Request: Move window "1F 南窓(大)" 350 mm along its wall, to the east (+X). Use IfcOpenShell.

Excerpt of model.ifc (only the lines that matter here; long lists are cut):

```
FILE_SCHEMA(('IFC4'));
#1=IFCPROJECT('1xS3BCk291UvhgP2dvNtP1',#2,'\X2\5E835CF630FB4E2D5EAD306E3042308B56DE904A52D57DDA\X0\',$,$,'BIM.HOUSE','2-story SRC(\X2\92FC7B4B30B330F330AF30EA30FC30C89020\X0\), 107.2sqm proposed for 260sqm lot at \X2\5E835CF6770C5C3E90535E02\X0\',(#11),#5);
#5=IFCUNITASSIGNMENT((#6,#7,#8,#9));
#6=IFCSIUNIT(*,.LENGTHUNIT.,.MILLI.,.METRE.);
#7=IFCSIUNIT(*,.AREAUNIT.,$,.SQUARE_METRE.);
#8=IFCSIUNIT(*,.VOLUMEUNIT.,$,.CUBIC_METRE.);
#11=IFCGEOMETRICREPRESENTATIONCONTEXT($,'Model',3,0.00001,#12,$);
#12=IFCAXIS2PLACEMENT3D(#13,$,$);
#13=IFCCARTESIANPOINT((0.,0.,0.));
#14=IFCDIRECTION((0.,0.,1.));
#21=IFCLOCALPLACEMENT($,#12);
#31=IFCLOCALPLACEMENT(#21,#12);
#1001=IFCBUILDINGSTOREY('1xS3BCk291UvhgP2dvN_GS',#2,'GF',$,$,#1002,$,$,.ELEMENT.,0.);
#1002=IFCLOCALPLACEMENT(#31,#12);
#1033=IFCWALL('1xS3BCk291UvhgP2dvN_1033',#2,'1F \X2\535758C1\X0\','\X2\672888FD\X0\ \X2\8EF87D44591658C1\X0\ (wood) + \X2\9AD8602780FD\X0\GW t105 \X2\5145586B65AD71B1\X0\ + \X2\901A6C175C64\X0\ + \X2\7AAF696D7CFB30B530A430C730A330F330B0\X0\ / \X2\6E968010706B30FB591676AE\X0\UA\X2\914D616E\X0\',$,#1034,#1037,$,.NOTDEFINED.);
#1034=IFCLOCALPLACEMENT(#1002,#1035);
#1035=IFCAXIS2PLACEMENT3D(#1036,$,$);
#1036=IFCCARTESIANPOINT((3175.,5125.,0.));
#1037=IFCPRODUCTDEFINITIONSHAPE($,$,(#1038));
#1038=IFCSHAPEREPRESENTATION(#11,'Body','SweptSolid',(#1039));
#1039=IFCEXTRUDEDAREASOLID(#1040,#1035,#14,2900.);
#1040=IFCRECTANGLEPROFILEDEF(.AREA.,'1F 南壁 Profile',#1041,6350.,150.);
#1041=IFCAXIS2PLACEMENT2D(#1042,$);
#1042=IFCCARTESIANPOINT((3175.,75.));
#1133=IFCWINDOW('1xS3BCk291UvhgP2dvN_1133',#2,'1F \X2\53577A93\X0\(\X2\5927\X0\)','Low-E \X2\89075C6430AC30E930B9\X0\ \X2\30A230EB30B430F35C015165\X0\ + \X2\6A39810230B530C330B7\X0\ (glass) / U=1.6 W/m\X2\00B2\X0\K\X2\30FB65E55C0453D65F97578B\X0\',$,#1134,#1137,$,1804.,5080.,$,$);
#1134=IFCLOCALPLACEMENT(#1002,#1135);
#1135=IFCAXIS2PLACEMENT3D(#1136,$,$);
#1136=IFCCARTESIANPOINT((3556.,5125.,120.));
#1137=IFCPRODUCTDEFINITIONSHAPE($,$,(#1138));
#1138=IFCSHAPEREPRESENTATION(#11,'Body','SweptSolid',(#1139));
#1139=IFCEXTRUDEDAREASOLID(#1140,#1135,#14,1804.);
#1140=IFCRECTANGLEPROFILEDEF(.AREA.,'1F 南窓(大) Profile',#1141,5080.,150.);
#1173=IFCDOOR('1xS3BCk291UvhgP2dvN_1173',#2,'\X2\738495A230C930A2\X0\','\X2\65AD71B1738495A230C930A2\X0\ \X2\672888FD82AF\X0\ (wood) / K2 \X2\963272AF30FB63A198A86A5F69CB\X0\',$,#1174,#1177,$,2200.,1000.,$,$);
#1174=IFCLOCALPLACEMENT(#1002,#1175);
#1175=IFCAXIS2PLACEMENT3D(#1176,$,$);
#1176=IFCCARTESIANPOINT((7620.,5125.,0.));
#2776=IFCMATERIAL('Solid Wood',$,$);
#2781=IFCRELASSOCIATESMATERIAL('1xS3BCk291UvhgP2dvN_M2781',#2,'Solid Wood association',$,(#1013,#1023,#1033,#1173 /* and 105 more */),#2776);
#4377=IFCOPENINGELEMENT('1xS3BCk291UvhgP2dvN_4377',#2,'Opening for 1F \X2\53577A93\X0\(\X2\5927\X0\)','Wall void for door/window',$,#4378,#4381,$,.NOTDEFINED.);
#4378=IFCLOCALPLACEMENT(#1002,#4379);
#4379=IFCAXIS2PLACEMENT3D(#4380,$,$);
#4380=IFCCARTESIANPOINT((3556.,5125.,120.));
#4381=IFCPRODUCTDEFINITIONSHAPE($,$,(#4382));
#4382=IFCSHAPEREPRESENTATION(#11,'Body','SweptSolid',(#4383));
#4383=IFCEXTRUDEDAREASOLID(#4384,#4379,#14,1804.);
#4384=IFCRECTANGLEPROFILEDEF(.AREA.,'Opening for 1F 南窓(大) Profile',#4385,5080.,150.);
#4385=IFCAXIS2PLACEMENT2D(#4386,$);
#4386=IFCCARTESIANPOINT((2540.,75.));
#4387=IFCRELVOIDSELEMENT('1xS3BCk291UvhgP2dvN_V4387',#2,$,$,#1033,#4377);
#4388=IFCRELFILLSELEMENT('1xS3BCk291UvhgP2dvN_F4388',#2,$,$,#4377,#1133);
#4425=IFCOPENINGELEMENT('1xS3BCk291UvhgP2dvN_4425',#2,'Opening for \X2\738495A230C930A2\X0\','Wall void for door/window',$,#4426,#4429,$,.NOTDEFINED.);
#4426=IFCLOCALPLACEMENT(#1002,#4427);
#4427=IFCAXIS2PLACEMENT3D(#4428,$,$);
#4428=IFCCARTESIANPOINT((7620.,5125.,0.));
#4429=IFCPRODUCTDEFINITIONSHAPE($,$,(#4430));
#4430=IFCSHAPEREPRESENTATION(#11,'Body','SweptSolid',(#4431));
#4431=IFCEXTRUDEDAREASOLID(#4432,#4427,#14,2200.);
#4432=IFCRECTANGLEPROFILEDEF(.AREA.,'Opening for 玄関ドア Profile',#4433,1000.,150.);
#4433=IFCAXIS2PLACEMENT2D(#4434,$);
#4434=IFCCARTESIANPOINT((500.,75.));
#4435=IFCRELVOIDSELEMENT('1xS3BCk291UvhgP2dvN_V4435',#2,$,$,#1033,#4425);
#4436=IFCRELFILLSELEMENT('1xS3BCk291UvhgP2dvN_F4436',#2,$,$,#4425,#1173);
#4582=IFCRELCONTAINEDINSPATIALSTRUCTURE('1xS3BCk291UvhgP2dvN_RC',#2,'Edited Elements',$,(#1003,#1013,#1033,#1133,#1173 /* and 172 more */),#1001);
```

```python
import ifcopenshell
import ifcopenshell.api.geometry
import ifcopenshell.util.placement
import ifcopenshell.util.unit

model = ifcopenshell.open("model.ifc")
unit_scale = ifcopenshell.util.unit.calculate_unit_scale(model)

window = model.by_id(1133)
opening = window.FillsVoids[0].RelatingOpeningElement
wall = opening.VoidsElements[0].RelatingBuildingElement

wall_matrix = ifcopenshell.util.placement.get_local_placement(wall.ObjectPlacement)
shift = wall_matrix[:3, 0] * 0.35 / unit_scale
before = ifcopenshell.util.placement.get_local_placement(window.ObjectPlacement)[:3, 3].copy()

# The window is not placed relative to its opening, so move both.
for product in (opening, window):
    matrix = ifcopenshell.util.placement.get_local_placement(product.ObjectPlacement)
    matrix[:3, 3] += shift
    ifcopenshell.api.geometry.edit_object_placement(model, product=product, matrix=matrix, is_si=False)

after = ifcopenshell.util.placement.get_local_placement(window.ObjectPlacement)[:3, 3]
print("window moved by", (after - before).round(3) + 0.0)

model.write("model_v2.ifc")
```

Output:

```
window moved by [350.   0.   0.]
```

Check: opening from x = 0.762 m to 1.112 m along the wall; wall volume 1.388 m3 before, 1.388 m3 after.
